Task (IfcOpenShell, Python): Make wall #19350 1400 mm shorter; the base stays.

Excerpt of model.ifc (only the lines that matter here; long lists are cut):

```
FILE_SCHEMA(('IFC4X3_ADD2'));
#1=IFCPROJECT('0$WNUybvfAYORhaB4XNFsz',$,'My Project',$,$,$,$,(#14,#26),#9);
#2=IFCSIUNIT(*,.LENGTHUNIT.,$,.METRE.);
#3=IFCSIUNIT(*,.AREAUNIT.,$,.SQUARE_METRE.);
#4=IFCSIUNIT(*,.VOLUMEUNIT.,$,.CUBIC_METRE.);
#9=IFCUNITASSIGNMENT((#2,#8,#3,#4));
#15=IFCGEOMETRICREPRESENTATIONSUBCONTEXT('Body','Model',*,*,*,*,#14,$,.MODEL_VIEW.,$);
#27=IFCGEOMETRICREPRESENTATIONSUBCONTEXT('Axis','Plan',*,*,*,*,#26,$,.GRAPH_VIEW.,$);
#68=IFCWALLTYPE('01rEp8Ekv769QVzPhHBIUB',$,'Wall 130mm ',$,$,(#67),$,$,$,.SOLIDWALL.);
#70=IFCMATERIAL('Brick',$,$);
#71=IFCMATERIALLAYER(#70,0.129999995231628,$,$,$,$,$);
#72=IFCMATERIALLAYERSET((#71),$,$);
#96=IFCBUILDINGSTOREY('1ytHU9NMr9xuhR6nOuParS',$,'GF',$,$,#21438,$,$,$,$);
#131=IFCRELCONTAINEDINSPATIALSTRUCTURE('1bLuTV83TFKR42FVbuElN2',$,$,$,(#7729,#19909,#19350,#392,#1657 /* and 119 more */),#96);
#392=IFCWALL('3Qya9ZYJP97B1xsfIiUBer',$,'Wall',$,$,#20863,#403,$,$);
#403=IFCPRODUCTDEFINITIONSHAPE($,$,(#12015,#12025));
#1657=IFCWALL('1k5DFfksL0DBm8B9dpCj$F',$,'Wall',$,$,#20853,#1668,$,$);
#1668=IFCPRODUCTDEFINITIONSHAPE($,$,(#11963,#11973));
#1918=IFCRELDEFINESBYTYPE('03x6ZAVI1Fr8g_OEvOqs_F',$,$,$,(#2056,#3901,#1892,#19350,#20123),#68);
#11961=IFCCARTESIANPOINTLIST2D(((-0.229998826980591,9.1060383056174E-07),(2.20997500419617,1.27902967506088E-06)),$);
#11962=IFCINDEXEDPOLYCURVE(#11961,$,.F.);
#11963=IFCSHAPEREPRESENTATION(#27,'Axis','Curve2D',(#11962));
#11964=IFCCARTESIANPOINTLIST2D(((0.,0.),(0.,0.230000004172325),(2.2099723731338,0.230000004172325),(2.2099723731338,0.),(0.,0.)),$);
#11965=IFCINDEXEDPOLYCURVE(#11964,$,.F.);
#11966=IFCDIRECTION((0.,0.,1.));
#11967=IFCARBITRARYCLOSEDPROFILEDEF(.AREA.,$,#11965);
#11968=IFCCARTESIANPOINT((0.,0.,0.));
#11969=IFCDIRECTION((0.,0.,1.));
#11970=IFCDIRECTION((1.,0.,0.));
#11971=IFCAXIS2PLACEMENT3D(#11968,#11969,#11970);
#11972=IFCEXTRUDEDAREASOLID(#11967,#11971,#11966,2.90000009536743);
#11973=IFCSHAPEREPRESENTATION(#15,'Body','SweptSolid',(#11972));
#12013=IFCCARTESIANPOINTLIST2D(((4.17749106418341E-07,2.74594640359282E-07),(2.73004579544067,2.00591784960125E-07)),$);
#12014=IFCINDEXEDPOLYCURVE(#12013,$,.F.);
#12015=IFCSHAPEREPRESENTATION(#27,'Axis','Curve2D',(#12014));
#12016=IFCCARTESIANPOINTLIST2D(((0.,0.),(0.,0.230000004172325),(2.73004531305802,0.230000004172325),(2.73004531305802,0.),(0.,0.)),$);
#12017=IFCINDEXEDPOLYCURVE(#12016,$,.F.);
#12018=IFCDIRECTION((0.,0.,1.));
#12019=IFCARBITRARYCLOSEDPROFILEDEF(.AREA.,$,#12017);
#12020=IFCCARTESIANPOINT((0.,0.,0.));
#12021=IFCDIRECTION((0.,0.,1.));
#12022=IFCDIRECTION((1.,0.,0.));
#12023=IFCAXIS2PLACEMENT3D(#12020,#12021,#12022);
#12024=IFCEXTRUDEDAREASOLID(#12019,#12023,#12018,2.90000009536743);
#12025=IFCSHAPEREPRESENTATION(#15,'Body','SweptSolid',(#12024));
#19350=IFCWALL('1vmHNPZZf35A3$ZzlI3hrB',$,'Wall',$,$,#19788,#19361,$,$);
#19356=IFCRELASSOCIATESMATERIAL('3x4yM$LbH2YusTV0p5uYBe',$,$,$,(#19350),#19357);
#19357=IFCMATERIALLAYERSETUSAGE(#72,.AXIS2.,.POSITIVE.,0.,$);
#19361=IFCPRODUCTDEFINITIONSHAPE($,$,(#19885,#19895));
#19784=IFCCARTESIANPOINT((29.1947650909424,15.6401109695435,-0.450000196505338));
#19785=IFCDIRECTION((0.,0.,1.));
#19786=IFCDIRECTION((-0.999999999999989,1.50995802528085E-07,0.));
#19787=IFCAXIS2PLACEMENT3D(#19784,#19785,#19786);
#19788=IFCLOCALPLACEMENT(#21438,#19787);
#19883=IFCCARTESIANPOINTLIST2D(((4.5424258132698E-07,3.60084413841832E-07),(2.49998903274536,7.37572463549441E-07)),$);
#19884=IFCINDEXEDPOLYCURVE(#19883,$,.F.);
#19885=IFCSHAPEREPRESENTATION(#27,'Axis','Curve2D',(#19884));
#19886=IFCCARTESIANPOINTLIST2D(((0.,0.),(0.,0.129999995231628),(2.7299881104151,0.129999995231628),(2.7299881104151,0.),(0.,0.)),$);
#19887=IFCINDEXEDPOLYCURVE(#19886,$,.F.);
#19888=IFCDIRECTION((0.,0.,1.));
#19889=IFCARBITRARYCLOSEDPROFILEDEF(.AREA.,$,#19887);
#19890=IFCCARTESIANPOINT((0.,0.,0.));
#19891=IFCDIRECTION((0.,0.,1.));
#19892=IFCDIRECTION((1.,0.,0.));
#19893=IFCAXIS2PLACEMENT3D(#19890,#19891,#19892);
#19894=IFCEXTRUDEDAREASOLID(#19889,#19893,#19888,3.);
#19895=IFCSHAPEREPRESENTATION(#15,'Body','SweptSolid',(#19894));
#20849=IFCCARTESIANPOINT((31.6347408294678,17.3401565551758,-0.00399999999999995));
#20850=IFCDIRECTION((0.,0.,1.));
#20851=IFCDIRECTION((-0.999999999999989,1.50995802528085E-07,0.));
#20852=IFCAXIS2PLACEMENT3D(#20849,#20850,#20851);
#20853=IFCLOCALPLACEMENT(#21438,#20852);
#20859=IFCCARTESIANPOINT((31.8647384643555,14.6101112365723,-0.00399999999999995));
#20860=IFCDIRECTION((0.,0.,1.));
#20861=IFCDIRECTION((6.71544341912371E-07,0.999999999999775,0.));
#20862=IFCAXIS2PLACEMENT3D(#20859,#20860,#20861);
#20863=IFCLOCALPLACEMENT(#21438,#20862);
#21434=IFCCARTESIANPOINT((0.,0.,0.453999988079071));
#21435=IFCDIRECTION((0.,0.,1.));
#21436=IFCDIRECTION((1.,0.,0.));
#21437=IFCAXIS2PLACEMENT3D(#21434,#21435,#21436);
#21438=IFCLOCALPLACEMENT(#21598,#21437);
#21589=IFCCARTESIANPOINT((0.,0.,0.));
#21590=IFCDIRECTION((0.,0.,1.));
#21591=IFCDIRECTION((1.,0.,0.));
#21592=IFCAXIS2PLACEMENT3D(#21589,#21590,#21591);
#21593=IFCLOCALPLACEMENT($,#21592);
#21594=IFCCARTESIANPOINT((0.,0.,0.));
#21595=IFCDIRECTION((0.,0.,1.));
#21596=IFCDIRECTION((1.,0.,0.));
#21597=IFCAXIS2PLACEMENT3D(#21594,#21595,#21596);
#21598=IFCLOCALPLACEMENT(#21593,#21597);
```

```python
import ifcopenshell
import ifcopenshell.geom
import ifcopenshell.util.representation
import ifcopenshell.util.shape
import ifcopenshell.util.unit

model = ifcopenshell.open("model.ifc")
unit_scale = ifcopenshell.util.unit.calculate_unit_scale(model)
settings = ifcopenshell.geom.settings()


def volume(element):
    """Net volume in cubic metres, openings subtracted."""
    shape = ifcopenshell.geom.create_shape(settings, element)
    return ifcopenshell.util.shape.get_volume(shape.geometry)


wall = model.by_id(19350)
before = volume(wall)

body = ifcopenshell.util.representation.get_representation(wall, "Model", "Body")
solid = body.Items[0]
old_height = solid.Depth
solid.Depth -= 1.4 / unit_scale
after = volume(wall)

print(f"height {old_height:g} -> {solid.Depth:g}, volume {before:.3f} -> {after:.3f} m3")

model.write("model_edited.ifc")
```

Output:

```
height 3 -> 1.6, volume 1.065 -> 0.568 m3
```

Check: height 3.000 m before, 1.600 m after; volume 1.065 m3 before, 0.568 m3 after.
